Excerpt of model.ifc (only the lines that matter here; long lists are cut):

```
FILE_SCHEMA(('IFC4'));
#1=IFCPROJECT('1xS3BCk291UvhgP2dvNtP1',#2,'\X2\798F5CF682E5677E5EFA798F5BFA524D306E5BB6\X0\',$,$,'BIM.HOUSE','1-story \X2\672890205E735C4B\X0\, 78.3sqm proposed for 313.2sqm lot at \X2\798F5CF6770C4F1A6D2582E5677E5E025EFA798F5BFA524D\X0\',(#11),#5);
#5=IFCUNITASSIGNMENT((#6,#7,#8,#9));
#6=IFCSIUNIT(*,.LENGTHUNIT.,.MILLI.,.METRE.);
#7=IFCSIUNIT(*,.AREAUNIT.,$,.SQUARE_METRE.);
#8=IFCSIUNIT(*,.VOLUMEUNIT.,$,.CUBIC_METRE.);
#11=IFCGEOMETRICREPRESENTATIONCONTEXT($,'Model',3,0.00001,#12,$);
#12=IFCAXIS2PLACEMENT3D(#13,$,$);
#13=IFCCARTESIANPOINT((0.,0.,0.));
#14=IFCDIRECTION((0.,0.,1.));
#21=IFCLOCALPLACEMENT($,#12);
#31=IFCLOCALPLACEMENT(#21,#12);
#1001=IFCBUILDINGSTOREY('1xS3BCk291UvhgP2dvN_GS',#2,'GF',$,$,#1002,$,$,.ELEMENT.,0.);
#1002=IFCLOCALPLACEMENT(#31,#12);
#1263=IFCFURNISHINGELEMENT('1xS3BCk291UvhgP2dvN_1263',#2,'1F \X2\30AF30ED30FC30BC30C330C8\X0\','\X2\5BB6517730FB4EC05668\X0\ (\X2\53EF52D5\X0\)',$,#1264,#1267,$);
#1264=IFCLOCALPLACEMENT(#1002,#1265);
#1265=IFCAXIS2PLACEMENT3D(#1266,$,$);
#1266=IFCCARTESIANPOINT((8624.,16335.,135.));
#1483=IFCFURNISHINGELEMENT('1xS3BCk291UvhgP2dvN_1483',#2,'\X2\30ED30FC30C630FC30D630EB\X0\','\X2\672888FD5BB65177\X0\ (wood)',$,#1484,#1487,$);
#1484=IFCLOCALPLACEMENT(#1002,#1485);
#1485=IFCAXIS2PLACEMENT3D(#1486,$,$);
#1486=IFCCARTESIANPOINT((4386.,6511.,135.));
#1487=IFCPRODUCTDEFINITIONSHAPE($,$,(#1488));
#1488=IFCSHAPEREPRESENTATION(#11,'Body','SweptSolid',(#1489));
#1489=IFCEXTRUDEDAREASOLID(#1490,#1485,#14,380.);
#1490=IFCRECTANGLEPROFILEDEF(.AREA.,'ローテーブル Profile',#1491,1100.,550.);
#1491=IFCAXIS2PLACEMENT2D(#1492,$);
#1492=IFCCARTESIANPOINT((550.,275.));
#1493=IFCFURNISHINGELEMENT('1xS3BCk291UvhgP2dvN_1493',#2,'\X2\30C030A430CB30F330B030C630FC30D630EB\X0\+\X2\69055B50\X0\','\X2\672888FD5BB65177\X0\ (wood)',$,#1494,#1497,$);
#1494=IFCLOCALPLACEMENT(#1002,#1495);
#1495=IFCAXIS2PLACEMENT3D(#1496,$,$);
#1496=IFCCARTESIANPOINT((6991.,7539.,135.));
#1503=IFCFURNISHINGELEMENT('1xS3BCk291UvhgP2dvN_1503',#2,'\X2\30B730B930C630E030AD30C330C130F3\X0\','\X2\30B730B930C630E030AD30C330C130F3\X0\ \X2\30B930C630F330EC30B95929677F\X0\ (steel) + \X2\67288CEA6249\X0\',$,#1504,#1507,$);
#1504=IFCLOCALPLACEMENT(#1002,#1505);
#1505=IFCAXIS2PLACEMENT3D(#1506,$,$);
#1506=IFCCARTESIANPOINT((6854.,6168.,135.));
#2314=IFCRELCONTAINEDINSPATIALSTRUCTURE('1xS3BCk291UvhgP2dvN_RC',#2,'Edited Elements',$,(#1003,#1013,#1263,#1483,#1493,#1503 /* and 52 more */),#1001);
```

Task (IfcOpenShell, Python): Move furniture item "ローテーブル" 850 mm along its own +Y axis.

```python
import ifcopenshell
import ifcopenshell.api.geometry
import ifcopenshell.util.placement
import ifcopenshell.util.unit

model = ifcopenshell.open("model.ifc")
unit_scale = ifcopenshell.util.unit.calculate_unit_scale(model)

item = model.by_guid("1xS3BCk291UvhgP2dvN_1483")
matrix = ifcopenshell.util.placement.get_local_placement(item.ObjectPlacement)
matrix[:3, 3] += matrix[:3, 1] * 0.85 / unit_scale
ifcopenshell.api.geometry.edit_object_placement(model, product=item, matrix=matrix, is_si=False)

print(ifcopenshell.util.placement.get_local_placement(item.ObjectPlacement).round(3) + 0.0)

model.write("model_updated.ifc")
```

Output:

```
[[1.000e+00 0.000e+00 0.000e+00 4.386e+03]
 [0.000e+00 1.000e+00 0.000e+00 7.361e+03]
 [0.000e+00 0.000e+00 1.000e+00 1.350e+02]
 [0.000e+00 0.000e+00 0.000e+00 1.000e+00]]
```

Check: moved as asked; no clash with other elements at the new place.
